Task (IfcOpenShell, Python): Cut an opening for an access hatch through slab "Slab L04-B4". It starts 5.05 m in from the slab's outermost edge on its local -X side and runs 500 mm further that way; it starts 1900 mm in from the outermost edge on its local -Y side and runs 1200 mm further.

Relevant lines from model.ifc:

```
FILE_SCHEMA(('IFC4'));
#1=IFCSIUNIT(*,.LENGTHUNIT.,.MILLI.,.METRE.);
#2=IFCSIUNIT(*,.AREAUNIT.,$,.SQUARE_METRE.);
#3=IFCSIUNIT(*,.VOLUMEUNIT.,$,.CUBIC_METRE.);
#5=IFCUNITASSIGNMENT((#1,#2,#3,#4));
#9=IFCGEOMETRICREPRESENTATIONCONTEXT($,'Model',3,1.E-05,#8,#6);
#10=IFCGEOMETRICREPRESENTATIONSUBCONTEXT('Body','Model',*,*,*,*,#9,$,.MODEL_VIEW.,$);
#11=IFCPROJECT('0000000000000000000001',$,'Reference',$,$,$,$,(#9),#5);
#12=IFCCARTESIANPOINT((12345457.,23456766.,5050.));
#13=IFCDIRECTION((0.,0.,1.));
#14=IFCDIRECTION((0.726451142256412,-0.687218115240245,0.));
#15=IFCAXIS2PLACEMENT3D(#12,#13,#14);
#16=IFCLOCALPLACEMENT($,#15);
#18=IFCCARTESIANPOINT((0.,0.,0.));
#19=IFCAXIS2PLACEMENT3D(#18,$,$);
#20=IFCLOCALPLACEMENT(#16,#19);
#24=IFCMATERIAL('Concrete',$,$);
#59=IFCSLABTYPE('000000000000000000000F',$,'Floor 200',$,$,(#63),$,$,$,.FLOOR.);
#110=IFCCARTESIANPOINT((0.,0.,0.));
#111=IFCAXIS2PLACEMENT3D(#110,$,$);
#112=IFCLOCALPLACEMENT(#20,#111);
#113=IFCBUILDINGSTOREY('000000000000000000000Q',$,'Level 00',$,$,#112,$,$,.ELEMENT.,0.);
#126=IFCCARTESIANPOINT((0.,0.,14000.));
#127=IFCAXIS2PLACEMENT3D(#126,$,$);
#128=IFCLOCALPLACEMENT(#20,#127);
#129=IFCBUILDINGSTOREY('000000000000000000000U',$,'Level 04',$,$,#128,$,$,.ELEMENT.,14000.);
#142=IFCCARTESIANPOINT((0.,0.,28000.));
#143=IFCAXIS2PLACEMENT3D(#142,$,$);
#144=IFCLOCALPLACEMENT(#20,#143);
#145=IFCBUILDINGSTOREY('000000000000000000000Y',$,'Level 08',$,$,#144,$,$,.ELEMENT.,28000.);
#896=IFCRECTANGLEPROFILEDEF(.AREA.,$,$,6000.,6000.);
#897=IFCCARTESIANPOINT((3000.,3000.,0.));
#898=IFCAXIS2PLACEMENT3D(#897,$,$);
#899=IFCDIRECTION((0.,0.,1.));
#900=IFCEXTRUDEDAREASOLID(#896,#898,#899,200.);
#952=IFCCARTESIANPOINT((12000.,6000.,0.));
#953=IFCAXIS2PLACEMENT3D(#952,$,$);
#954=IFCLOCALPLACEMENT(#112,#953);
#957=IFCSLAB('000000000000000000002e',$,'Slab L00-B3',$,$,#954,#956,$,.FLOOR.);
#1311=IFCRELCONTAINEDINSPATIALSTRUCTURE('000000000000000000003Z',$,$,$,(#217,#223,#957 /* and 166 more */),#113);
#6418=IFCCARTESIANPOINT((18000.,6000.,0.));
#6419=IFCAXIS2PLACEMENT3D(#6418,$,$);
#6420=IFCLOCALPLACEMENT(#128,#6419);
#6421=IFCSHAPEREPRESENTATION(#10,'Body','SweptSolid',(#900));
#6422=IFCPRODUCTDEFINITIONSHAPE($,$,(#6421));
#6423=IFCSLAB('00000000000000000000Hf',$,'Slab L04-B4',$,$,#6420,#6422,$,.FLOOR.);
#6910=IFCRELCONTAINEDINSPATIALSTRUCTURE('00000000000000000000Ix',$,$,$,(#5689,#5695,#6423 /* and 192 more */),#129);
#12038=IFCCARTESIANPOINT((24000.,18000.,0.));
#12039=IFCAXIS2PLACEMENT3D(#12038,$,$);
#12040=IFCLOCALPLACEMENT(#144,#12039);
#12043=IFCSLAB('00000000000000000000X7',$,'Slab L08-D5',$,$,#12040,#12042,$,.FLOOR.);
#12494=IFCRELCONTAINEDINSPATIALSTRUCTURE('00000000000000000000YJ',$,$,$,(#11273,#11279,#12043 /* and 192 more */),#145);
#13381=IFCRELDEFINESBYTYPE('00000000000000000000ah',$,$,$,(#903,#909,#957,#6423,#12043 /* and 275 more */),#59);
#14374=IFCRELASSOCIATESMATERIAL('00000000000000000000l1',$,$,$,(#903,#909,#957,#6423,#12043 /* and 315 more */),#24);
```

```python
import numpy as np
import ifcopenshell
import ifcopenshell.api.feature
import ifcopenshell.api.geometry
import ifcopenshell.api.root
import ifcopenshell.geom
import ifcopenshell.util.placement
import ifcopenshell.util.representation
import ifcopenshell.util.shape
import ifcopenshell.util.unit

model = ifcopenshell.open("model.ifc")
unit_scale = ifcopenshell.util.unit.calculate_unit_scale(model)
settings = ifcopenshell.geom.settings()


def volume(element):
    """Net volume in cubic metres, openings subtracted."""
    shape = ifcopenshell.geom.create_shape(settings, element)
    return ifcopenshell.util.shape.get_volume(shape.geometry)


slab = model.by_guid("00000000000000000000Hf")
before = volume(slab)

# Extent in the slab's own axes, in metres. The edges named are its -X and -Y sides.
slab_shape = ifcopenshell.geom.create_shape(settings, slab)
vertices = ifcopenshell.util.shape.get_vertices(slab_shape.geometry)
x_min, y_min, bottom = vertices.min(axis=0)
top = vertices[:, 2].max()

opening = ifcopenshell.api.root.create_entity(model, ifc_class="IfcOpeningElement", name="Access hatch opening", predefined_type="OPENING")
context = ifcopenshell.util.representation.get_context(model, "Model", "Body", "MODEL_VIEW")
width, depth = 0.5, 1.2
outline = [(0.0, 0.0), (width, 0.0), (width, depth), (0.0, depth), (0.0, 0.0)]
# Overshoot both faces by 50 mm so the cut is clean.
shape = ifcopenshell.api.geometry.add_slab_representation(
    model, context=context, depth=top - bottom + 0.1, polyline=outline
)
ifcopenshell.api.geometry.assign_representation(model, product=opening, representation=shape)

matrix = ifcopenshell.util.placement.get_local_placement(slab.ObjectPlacement)
matrix[:, 3] = matrix @ np.append(np.array([x_min + 5.05, y_min + 1.9, bottom - 0.05]) / unit_scale, 1.0)
ifcopenshell.api.geometry.edit_object_placement(model, product=opening, matrix=matrix, is_si=False)
ifcopenshell.api.feature.add_feature(model, feature=opening, element=slab)

after = volume(slab)

print(f"slab volume {before:.3f} -> {after:.3f} m3")

model.write("model_edited.ifc")
```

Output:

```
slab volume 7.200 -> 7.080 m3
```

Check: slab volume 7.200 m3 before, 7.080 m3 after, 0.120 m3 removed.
